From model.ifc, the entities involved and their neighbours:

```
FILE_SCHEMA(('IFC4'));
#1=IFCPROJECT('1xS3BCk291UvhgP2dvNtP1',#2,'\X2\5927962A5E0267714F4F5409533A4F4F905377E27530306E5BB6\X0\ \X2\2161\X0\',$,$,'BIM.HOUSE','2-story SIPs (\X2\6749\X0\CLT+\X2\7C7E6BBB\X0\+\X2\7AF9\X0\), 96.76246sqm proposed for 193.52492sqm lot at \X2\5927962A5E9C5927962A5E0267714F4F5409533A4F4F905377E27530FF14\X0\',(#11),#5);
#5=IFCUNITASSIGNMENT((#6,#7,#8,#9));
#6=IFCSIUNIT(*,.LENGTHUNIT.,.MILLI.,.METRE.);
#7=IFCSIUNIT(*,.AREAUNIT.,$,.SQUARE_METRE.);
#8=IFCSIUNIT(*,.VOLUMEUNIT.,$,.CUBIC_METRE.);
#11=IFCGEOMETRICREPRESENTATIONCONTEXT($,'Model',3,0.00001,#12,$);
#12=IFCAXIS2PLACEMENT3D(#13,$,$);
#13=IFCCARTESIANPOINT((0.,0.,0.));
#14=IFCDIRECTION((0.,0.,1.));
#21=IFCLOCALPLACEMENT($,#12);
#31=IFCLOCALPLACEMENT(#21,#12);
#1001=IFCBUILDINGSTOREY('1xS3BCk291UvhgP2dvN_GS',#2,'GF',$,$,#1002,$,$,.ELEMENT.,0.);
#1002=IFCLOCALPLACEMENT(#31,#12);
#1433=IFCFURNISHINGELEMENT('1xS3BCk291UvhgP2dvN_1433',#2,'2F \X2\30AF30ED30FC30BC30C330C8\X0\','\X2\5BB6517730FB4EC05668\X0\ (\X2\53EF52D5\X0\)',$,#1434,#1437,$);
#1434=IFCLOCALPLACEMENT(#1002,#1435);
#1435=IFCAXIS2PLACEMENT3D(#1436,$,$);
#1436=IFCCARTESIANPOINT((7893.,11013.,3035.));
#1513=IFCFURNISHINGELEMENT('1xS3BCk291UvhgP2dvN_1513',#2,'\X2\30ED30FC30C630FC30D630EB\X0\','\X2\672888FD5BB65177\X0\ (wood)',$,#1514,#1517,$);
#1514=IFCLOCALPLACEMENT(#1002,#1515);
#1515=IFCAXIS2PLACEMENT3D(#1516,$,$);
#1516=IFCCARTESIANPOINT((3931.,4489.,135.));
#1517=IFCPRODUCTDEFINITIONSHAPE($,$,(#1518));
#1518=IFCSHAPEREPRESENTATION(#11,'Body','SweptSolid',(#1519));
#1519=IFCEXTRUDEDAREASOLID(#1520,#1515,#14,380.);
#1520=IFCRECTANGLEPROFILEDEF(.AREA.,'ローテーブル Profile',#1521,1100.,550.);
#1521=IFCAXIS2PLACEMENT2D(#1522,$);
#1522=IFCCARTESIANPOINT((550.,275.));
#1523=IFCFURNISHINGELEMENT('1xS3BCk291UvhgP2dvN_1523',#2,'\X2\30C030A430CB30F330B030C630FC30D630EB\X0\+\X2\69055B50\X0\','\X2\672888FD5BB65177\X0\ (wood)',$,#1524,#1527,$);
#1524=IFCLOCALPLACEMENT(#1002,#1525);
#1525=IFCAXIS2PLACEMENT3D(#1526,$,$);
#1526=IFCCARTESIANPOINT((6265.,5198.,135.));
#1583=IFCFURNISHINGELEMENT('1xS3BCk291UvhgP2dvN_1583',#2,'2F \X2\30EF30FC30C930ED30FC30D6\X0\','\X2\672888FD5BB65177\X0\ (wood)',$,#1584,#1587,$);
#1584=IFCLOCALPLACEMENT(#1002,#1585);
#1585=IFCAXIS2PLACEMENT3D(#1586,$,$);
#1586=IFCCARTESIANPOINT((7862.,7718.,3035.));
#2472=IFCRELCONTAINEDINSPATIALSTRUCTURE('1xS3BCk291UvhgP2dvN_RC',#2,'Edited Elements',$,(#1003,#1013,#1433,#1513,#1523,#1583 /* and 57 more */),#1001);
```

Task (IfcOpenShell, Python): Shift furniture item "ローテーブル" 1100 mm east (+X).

```python
import ifcopenshell
import ifcopenshell.api.geometry
import ifcopenshell.util.placement

model = ifcopenshell.open("model.ifc")

item = model.by_guid("1xS3BCk291UvhgP2dvN_1513")
matrix = ifcopenshell.util.placement.get_local_placement(item.ObjectPlacement)
matrix[0, 3] += 1100.0
ifcopenshell.api.geometry.edit_object_placement(model, product=item, matrix=matrix, is_si=False)

print(ifcopenshell.util.placement.get_local_placement(item.ObjectPlacement).round(3) + 0.0)

model.write("model_v2.ifc")
```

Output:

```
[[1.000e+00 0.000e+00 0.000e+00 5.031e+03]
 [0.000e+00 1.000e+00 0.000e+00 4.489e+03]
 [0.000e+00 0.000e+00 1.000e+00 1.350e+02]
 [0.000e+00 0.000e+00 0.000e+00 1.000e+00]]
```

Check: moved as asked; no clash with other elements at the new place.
